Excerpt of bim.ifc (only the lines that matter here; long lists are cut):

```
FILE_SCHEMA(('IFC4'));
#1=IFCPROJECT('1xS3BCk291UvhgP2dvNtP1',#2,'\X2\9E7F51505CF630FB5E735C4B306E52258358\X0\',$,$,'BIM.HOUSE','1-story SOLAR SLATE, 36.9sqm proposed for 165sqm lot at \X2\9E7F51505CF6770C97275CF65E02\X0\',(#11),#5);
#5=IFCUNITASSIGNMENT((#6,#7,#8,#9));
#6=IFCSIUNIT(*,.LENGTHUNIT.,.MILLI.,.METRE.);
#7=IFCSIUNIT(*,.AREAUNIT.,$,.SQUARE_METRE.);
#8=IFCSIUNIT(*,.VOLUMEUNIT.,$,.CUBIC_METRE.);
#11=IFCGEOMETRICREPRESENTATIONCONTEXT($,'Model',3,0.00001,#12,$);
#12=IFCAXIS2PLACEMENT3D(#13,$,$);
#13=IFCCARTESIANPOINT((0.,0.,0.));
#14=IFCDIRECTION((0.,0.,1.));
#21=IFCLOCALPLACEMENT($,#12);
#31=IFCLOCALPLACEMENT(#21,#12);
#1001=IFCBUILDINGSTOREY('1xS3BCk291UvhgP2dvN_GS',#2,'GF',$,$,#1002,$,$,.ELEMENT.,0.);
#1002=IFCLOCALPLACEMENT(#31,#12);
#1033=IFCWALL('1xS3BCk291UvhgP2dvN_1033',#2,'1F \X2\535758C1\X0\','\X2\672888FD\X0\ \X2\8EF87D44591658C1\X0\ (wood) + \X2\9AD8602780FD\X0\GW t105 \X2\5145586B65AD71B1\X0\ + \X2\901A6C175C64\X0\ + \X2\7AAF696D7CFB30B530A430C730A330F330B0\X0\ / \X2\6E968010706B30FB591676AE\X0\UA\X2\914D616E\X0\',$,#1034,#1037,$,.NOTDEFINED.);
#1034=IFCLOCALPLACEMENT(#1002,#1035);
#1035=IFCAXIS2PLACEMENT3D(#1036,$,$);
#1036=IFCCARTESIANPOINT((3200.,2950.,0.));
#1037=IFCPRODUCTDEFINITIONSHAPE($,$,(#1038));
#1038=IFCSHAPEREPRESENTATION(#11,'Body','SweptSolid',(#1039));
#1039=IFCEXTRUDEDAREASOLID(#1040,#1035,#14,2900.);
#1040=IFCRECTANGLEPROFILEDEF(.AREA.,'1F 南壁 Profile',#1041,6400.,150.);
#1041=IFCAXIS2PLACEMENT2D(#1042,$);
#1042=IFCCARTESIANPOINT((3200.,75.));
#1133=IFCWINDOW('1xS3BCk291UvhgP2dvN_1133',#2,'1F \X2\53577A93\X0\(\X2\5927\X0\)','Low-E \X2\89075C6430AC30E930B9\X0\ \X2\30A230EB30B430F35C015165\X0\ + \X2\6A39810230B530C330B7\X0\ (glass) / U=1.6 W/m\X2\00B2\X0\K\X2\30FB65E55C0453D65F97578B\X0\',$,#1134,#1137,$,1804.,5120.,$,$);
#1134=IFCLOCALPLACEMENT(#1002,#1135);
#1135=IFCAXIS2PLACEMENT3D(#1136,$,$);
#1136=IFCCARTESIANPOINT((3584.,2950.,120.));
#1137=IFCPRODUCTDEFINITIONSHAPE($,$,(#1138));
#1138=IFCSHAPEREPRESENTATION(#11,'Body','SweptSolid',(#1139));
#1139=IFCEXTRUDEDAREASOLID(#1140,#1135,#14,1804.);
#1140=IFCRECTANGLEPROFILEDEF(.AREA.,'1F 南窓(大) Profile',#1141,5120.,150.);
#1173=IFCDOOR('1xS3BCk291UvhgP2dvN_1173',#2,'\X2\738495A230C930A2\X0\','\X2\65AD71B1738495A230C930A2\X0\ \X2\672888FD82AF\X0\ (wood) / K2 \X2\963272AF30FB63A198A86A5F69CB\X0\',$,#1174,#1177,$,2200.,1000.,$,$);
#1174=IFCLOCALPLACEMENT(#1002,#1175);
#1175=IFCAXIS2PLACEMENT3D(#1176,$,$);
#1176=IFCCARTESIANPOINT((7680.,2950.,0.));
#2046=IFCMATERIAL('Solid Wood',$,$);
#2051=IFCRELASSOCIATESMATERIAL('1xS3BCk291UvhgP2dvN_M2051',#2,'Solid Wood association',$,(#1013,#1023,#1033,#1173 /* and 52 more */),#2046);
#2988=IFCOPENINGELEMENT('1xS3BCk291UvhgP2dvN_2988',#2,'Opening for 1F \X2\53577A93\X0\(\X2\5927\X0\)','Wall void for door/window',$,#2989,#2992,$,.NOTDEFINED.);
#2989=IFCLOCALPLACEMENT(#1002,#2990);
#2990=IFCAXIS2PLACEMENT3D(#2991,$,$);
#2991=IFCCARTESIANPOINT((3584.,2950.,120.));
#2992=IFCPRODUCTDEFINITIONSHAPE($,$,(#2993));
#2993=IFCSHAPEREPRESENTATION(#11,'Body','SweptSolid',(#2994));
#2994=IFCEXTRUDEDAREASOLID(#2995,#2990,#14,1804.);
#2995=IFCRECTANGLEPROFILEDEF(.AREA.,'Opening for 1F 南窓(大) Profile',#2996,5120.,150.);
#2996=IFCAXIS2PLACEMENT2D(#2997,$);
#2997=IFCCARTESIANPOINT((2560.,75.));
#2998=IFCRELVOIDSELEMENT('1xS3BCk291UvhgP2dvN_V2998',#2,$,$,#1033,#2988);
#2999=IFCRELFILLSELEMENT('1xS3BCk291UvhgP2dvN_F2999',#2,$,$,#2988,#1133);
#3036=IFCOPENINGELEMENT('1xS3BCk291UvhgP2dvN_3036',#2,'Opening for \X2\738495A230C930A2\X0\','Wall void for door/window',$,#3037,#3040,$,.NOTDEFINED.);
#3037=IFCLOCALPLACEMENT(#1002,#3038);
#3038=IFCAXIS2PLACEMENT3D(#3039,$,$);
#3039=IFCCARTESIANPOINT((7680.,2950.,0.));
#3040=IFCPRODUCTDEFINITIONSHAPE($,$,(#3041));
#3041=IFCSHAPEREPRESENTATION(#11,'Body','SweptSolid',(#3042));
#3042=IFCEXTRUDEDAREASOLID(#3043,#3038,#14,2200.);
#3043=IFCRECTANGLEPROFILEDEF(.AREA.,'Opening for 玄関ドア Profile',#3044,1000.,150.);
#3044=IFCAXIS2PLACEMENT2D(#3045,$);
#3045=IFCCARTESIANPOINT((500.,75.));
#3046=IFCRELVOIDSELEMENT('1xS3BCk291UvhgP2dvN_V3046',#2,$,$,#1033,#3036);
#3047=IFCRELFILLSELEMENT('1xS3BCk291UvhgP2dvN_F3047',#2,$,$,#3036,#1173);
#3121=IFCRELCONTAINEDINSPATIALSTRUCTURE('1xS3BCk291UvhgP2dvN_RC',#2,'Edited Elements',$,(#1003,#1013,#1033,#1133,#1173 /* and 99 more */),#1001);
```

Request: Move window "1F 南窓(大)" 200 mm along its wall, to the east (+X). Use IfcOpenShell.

```python
import ifcopenshell
import ifcopenshell.api.geometry
import ifcopenshell.util.placement
import ifcopenshell.util.unit

model = ifcopenshell.open("bim.ifc")
unit_scale = ifcopenshell.util.unit.calculate_unit_scale(model)

window = model.by_guid("1xS3BCk291UvhgP2dvN_1133")
opening = window.FillsVoids[0].RelatingOpeningElement
wall = opening.VoidsElements[0].RelatingBuildingElement

wall_matrix = ifcopenshell.util.placement.get_local_placement(wall.ObjectPlacement)
shift = wall_matrix[:3, 0] * 0.2 / unit_scale
before = ifcopenshell.util.placement.get_local_placement(window.ObjectPlacement)[:3, 3].copy()

# The window is not placed relative to its opening, so move both.
for product in (opening, window):
    matrix = ifcopenshell.util.placement.get_local_placement(product.ObjectPlacement)
    matrix[:3, 3] += shift
    ifcopenshell.api.geometry.edit_object_placement(model, product=product, matrix=matrix, is_si=False)

after = ifcopenshell.util.placement.get_local_placement(window.ObjectPlacement)[:3, 3]
print("window moved by", (after - before).round(3) + 0.0)

model.write("bim_edited.ifc")
```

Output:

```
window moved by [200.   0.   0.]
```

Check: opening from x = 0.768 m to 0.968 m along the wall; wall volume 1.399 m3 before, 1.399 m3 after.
